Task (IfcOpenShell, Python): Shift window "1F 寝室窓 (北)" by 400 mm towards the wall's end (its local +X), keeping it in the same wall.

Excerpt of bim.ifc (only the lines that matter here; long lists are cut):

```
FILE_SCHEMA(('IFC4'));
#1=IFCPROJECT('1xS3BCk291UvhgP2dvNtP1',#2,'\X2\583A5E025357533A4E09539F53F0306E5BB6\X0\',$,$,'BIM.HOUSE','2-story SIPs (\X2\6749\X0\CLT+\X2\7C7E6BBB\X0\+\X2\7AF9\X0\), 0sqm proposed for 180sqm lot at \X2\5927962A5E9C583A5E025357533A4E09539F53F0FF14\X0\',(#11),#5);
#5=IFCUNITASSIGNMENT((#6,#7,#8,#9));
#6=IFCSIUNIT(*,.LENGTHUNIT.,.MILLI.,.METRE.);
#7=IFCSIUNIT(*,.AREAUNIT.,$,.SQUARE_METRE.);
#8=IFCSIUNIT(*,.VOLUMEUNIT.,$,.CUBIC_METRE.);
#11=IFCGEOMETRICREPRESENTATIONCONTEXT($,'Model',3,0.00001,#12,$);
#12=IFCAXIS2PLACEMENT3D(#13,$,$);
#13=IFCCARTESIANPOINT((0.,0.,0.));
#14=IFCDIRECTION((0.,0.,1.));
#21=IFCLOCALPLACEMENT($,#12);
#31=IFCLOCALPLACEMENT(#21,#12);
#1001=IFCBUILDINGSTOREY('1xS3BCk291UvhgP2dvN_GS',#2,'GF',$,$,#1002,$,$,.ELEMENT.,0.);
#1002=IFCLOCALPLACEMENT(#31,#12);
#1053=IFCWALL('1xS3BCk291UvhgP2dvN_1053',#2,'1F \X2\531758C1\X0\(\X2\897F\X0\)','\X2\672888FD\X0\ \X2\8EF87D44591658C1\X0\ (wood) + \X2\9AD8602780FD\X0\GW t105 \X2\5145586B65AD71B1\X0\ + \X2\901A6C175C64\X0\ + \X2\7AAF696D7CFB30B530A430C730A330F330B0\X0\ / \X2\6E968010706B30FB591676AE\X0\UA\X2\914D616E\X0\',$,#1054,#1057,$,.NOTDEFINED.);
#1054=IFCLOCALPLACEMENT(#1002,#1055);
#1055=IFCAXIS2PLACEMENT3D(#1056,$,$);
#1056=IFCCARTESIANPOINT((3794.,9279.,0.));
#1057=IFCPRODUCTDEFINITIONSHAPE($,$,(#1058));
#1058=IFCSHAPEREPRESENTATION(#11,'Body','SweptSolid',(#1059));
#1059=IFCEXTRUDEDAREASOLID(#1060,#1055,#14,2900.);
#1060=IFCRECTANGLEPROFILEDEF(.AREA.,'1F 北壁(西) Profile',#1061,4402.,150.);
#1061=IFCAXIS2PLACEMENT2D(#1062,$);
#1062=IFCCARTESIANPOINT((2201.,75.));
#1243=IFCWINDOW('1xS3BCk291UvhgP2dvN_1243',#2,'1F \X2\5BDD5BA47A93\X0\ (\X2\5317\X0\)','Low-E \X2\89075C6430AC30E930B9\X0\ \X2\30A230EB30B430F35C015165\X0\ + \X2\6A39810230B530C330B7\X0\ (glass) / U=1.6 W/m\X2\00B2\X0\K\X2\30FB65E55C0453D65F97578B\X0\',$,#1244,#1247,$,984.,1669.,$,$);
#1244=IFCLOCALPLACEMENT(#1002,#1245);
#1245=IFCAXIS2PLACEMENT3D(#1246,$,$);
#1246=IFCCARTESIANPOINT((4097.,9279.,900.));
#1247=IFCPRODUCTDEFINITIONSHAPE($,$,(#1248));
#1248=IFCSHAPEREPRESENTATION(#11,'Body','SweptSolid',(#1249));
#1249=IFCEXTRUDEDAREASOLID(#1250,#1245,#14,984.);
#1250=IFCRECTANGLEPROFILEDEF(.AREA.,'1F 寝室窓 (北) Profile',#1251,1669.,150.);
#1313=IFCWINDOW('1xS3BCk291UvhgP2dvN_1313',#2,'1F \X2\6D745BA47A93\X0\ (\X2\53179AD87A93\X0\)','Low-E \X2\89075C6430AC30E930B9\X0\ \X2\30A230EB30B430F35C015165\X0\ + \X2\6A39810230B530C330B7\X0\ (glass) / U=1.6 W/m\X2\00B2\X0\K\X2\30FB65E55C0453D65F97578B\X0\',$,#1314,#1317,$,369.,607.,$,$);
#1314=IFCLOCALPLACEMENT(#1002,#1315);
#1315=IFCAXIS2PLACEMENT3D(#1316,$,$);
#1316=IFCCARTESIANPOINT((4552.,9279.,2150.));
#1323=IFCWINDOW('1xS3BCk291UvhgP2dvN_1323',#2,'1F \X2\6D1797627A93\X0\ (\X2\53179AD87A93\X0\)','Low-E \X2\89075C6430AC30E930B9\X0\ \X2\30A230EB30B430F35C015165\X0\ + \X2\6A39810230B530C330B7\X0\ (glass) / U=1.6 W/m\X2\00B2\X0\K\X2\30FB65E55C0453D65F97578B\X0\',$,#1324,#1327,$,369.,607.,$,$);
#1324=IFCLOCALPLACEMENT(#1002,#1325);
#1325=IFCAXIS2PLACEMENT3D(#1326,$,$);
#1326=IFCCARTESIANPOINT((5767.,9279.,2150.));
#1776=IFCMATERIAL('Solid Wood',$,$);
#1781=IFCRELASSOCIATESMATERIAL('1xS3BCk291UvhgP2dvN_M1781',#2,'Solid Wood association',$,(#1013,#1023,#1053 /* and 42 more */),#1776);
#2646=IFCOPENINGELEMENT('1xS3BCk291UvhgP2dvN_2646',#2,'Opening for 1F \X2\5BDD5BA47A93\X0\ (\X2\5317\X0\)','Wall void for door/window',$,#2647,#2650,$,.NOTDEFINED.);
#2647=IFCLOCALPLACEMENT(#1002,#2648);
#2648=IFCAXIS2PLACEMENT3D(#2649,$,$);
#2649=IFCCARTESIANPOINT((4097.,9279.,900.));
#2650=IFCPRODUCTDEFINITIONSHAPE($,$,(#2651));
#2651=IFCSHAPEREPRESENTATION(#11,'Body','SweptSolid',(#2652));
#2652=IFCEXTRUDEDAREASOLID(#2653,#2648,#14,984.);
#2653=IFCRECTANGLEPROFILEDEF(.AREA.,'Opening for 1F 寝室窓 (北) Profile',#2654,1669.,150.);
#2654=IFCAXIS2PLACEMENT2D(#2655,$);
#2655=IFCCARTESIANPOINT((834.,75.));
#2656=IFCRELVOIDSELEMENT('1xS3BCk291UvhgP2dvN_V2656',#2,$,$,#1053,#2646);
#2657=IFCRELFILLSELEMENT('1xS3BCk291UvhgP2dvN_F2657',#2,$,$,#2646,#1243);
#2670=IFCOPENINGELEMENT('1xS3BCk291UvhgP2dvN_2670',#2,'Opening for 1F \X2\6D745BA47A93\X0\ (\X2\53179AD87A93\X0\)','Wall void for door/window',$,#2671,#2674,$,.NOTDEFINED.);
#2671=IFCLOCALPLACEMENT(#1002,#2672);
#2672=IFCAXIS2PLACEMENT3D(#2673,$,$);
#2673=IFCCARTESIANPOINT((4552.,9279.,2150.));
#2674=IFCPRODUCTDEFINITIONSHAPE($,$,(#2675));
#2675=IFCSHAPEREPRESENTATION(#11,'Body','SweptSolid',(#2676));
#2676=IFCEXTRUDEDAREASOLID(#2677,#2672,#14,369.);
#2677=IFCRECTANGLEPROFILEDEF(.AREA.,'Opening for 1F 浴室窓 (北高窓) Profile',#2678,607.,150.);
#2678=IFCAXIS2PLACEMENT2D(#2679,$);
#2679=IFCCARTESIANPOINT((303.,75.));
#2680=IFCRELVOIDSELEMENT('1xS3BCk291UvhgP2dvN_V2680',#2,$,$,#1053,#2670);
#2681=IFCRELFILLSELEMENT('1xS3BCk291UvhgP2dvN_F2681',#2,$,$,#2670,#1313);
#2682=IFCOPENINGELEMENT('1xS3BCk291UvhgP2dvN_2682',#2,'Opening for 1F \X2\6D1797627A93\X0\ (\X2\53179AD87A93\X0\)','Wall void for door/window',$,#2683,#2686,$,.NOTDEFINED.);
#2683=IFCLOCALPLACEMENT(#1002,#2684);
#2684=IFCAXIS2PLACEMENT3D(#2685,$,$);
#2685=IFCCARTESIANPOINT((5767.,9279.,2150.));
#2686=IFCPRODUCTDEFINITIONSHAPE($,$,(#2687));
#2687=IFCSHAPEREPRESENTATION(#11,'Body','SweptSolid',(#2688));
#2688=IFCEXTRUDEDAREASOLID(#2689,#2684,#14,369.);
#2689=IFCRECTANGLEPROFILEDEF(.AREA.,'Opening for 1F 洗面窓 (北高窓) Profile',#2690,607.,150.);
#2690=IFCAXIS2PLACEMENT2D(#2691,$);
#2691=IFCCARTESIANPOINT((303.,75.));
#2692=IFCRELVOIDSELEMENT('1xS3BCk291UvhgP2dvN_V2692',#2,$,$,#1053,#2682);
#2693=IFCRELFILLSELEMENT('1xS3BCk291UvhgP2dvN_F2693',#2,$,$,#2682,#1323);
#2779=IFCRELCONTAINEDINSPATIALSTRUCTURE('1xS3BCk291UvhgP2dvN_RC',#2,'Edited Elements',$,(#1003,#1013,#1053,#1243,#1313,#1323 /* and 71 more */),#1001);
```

```python
import ifcopenshell
import ifcopenshell.api.geometry
import ifcopenshell.util.placement
import ifcopenshell.util.unit

model = ifcopenshell.open("bim.ifc")
unit_scale = ifcopenshell.util.unit.calculate_unit_scale(model)

window = model.by_guid("1xS3BCk291UvhgP2dvN_1243")
opening = window.FillsVoids[0].RelatingOpeningElement
wall = opening.VoidsElements[0].RelatingBuildingElement

wall_matrix = ifcopenshell.util.placement.get_local_placement(wall.ObjectPlacement)
shift = wall_matrix[:3, 0] * 0.4 / unit_scale
before = ifcopenshell.util.placement.get_local_placement(window.ObjectPlacement)[:3, 3].copy()

# The window is not placed relative to its opening, so move both.
for product in (opening, window):
    matrix = ifcopenshell.util.placement.get_local_placement(product.ObjectPlacement)
    matrix[:3, 3] += shift
    ifcopenshell.api.geometry.edit_object_placement(model, product=product, matrix=matrix, is_si=False)

after = ifcopenshell.util.placement.get_local_placement(window.ObjectPlacement)[:3, 3]
print("window moved by", (after - before).round(3) + 0.0)

model.write("bim_updated.ifc")
```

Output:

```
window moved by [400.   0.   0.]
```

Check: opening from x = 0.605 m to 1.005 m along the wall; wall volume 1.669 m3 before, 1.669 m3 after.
